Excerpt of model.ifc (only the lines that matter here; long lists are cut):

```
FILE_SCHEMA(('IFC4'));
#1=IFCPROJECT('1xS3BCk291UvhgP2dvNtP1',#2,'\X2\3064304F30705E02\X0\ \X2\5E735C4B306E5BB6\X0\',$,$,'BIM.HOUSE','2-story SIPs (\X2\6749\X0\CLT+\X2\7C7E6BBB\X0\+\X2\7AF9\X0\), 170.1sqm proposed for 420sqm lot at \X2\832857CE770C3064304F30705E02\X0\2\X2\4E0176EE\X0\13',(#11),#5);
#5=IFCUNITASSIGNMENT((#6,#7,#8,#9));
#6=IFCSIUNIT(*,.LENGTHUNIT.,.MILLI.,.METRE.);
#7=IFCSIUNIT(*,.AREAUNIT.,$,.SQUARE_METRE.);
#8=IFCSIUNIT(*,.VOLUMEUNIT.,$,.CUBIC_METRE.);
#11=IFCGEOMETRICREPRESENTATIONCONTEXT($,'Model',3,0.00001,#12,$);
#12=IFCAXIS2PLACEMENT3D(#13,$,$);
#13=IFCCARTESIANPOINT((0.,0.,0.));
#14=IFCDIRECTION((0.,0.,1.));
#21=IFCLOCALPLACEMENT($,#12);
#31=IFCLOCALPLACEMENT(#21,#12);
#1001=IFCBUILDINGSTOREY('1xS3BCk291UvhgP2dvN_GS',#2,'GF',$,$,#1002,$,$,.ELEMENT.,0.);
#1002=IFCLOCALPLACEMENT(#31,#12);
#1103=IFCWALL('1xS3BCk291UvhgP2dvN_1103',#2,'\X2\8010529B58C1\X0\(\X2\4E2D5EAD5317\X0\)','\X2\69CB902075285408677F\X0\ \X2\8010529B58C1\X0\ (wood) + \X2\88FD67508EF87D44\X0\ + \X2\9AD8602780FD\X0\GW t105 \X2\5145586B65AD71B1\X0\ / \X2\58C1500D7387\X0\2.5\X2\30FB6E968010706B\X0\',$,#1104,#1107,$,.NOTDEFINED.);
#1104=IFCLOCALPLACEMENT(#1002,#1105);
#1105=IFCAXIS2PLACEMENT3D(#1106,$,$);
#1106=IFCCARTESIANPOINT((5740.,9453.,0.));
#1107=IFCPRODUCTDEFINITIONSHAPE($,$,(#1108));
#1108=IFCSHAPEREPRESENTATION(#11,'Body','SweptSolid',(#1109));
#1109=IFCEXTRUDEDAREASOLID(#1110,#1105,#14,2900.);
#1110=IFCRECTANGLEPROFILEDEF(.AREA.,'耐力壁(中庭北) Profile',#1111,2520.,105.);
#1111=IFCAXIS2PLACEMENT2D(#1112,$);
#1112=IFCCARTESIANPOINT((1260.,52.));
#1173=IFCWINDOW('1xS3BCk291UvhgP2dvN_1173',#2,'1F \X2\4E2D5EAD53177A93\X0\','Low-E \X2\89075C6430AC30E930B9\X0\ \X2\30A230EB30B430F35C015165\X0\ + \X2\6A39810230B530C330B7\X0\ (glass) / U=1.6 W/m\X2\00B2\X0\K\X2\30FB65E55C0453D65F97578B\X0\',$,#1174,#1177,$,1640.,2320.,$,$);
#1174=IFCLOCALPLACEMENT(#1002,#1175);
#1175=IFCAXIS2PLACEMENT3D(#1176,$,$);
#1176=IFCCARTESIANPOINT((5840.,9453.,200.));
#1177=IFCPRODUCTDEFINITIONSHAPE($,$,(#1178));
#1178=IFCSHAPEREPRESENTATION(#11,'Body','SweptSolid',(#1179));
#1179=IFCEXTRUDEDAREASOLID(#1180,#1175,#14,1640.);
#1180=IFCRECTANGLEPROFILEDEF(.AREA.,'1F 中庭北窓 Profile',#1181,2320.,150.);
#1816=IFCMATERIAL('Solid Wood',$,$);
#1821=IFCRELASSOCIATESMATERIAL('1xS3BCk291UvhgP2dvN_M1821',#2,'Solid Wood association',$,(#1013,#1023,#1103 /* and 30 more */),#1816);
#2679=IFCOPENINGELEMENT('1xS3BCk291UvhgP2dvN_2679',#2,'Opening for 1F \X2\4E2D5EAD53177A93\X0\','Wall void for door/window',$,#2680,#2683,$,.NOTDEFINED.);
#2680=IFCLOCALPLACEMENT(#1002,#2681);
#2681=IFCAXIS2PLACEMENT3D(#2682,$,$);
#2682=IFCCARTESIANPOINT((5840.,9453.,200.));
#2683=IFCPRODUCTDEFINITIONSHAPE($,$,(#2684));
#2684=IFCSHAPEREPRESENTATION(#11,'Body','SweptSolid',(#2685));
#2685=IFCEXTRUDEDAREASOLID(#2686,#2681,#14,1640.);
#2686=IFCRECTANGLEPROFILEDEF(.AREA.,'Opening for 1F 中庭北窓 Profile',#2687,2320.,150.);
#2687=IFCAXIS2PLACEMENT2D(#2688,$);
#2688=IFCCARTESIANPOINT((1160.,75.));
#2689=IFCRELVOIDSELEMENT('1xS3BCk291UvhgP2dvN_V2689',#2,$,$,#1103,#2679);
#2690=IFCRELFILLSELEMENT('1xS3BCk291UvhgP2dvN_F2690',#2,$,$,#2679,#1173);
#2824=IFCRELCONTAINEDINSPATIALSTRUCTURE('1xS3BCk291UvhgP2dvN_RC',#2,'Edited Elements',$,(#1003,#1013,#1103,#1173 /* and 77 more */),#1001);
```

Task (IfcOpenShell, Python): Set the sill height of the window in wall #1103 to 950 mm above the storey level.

```python
import numpy as np
import ifcopenshell
import ifcopenshell.api.geometry
import ifcopenshell.geom
import ifcopenshell.util.element
import ifcopenshell.util.placement
import ifcopenshell.util.shape
import ifcopenshell.util.unit

model = ifcopenshell.open("model.ifc")
unit_scale = ifcopenshell.util.unit.calculate_unit_scale(model)

window = model.by_id(1173)
opening = window.FillsVoids[0].RelatingOpeningElement
storey = ifcopenshell.util.element.get_container(window, ifc_class="IfcBuildingStorey")
level = ifcopenshell.util.placement.get_local_placement(storey.ObjectPlacement)[2, 3]

# The opening's origin need not be at the sill, so measure its lowest point.
shape = ifcopenshell.geom.create_shape(ifcopenshell.geom.settings(), opening)
bottom = ifcopenshell.util.shape.get_shape_bottom_elevation(shape, shape.geometry) / unit_scale
dz = level + 0.95 / unit_scale - bottom

shift = np.array([0.0, 0.0, dz])
# The window is not placed relative to its opening, so move both.
for product in (opening, window):
    matrix = ifcopenshell.util.placement.get_local_placement(product.ObjectPlacement)
    matrix[:3, 3] += shift
    ifcopenshell.api.geometry.edit_object_placement(model, product=product, matrix=matrix, is_si=False)

print(f"moved by {dz * unit_scale:+.3f} m")

model.write("model_edited.ifc")
```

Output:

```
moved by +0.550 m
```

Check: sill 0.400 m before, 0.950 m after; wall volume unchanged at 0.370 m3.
